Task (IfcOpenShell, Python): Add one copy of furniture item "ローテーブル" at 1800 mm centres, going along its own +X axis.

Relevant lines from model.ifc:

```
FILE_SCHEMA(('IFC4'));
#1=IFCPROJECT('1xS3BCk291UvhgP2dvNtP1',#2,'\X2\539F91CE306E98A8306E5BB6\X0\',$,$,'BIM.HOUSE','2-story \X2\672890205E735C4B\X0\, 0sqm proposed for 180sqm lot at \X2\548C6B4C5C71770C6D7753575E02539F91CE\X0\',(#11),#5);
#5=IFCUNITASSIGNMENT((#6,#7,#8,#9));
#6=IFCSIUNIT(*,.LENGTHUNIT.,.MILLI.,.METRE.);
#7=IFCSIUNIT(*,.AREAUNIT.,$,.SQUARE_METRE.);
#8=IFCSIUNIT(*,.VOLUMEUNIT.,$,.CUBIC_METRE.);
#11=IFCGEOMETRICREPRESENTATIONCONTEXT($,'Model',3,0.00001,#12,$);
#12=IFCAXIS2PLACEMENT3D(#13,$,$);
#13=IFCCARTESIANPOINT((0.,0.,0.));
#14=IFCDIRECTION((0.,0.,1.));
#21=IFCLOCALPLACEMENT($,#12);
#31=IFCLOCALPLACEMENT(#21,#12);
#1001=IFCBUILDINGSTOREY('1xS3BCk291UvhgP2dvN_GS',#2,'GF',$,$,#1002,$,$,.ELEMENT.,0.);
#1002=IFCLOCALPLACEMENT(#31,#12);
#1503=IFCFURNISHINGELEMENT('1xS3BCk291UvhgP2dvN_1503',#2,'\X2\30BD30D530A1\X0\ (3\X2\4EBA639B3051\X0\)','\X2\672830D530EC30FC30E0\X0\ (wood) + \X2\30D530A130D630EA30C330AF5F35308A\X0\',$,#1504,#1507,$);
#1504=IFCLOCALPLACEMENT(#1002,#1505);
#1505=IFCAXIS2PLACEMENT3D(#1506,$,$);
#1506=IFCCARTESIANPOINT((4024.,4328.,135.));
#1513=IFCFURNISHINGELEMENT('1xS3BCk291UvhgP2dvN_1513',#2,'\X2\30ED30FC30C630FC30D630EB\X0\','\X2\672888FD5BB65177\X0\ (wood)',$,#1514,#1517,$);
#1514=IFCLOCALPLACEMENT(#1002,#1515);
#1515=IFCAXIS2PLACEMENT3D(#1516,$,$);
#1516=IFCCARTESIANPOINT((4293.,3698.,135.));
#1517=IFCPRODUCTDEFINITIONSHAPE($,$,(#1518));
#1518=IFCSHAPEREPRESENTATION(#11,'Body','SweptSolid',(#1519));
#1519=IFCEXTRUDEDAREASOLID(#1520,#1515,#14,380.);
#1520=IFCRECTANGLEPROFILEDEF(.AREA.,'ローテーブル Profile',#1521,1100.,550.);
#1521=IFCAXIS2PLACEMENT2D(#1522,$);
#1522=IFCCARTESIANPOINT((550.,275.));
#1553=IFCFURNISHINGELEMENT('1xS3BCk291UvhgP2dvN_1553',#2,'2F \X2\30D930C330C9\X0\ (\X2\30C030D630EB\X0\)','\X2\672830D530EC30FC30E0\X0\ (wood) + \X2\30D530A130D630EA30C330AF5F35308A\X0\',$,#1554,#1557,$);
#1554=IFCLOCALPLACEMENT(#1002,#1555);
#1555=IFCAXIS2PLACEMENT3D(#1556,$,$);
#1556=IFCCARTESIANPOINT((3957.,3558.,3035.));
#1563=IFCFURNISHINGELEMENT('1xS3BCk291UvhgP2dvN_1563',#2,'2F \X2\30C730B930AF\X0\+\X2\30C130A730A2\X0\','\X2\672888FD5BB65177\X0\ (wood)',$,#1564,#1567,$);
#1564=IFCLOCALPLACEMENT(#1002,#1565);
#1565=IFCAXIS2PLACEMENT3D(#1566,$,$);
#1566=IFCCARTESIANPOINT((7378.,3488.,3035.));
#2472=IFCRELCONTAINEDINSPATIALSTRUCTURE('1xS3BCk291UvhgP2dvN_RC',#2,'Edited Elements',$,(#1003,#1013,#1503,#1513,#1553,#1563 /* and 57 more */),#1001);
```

```python
import ifcopenshell
import ifcopenshell.api.geometry
import ifcopenshell.api.root
import ifcopenshell.util.element
import ifcopenshell.util.placement
import ifcopenshell.util.unit

model = ifcopenshell.open("model.ifc")
unit_scale = ifcopenshell.util.unit.calculate_unit_scale(model)


def reuse_history(source, copy):
    """copy_class also copies each property set's owner history, people and application; keep the originals."""
    for rel in copy.IsDefinedBy:
        if rel.is_a("IfcRelDefinesByProperties") and (history := rel.RelatingPropertyDefinition.OwnerHistory):
            rel.RelatingPropertyDefinition.OwnerHistory = source.OwnerHistory
            ifcopenshell.util.element.remove_deep2(model, history)


source = model.by_id(1513)
base = ifcopenshell.util.placement.get_local_placement(source.ObjectPlacement)
step = base[:3, 0] * 1.8 / unit_scale

for i in range(1, 2):
    copy = ifcopenshell.api.root.copy_class(model, product=source)
    copy.Representation = ifcopenshell.util.element.copy_deep(
        model, source.Representation, exclude=["IfcGeometricRepresentationContext", "IfcRepresentationMap"]
    )
    reuse_history(source, copy)
    matrix = base.copy()
    matrix[:3, 3] += i * step
    print("added at", matrix[:3, 3].round(3) + 0.0)
    ifcopenshell.api.geometry.edit_object_placement(model, product=copy, matrix=matrix, is_si=False)

model.write("model_v2.ifc")
```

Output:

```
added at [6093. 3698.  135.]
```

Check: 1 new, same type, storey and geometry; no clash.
